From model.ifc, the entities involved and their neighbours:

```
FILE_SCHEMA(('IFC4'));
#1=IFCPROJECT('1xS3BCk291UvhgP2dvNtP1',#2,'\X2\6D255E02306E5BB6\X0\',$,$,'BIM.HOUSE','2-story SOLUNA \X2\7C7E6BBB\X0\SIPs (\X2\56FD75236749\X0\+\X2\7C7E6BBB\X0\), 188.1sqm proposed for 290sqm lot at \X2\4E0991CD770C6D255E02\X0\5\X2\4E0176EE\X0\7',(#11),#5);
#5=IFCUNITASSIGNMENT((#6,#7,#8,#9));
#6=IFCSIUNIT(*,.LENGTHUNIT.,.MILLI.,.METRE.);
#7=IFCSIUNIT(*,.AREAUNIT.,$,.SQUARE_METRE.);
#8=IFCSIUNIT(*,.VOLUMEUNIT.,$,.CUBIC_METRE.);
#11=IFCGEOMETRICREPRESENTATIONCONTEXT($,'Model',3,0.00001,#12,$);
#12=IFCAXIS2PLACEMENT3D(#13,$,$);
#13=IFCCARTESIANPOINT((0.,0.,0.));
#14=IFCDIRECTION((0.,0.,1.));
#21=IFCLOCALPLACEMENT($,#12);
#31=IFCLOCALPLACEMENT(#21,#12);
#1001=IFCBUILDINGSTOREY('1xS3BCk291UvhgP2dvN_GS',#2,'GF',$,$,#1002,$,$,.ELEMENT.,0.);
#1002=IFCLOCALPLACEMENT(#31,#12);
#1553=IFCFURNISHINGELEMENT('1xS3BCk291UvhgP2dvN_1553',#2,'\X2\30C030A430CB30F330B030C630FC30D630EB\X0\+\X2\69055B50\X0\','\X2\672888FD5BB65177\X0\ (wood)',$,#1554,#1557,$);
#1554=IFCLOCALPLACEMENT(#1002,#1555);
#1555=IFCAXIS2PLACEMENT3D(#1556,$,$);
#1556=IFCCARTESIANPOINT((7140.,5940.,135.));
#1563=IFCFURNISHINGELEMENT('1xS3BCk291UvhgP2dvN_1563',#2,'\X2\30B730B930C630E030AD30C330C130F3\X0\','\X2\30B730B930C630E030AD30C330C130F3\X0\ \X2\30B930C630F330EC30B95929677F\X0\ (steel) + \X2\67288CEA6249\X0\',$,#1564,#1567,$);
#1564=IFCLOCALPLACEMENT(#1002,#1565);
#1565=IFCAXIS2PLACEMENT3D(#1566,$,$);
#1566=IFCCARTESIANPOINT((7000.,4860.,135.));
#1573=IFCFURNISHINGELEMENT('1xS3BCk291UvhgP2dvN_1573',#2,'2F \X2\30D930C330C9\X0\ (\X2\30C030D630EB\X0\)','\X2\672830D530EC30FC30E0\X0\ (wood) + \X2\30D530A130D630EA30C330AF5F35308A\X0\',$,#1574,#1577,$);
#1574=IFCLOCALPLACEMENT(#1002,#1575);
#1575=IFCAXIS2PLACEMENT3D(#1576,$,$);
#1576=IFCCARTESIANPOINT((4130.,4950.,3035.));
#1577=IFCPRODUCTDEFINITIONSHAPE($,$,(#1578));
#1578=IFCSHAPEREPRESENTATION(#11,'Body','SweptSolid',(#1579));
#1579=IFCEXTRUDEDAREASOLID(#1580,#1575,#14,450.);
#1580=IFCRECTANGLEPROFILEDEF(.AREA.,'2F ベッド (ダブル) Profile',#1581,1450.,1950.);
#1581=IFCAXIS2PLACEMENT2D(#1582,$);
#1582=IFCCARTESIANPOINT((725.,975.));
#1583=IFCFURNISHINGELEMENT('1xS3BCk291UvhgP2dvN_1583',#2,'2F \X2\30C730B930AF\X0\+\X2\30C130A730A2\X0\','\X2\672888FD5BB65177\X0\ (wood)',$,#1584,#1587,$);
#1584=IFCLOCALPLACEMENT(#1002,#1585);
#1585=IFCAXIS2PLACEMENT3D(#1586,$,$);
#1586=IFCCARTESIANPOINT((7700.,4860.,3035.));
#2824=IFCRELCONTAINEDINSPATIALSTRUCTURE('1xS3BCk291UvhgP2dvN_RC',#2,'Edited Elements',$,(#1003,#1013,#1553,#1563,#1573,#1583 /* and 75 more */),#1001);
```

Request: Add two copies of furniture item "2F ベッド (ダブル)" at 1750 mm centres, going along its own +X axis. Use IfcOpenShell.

```python
import ifcopenshell
import ifcopenshell.api.geometry
import ifcopenshell.api.root
import ifcopenshell.util.element
import ifcopenshell.util.placement

model = ifcopenshell.open("model.ifc")


def reuse_history(source, copy):
    """copy_class also copies each property set's owner history, people and application; keep the originals."""
    for rel in copy.IsDefinedBy:
        if rel.is_a("IfcRelDefinesByProperties") and (history := rel.RelatingPropertyDefinition.OwnerHistory):
            rel.RelatingPropertyDefinition.OwnerHistory = source.OwnerHistory
            ifcopenshell.util.element.remove_deep2(model, history)


source = model.by_guid("1xS3BCk291UvhgP2dvN_1573")
base = ifcopenshell.util.placement.get_local_placement(source.ObjectPlacement)
step = base[:3, 0] * 1750.0

for i in range(1, 3):
    copy = ifcopenshell.api.root.copy_class(model, product=source)
    copy.Representation = ifcopenshell.util.element.copy_deep(
        model, source.Representation, exclude=["IfcGeometricRepresentationContext", "IfcRepresentationMap"]
    )
    reuse_history(source, copy)
    matrix = base.copy()
    matrix[:3, 3] += i * step
    print("added at", matrix[:3, 3].round(3) + 0.0)
    ifcopenshell.api.geometry.edit_object_placement(model, product=copy, matrix=matrix, is_si=False)

model.write("model_edited.ifc")
```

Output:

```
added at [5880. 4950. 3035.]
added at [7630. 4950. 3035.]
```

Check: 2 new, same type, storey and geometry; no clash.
